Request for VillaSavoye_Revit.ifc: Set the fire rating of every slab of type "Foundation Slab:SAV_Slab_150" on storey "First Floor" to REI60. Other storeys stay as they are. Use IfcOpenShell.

First a look at what the model holds.

```python
import ifcopenshell
import ifcopenshell.util.element

model = ifcopenshell.open("VillaSavoye_Revit.ifc")
print(model.schema)
storey = next(s for s in model.by_type("IfcBuildingStorey") if s.Name == "First Floor")
slabs = [e for e in ifcopenshell.util.element.get_decomposition(storey) if e.is_a("IfcSlab")]
seen = {}
for e in slabs:
    element_type = ifcopenshell.util.element.get_type(e)
    key = (element_type.Name if element_type != e and element_type else None, ifcopenshell.util.element.get_pset(e, "Pset_SlabCommon", "FireRating"))
    seen[key] = seen.get(key, 0) + 1
for (name, value), count in sorted(seen.items(), key=str):
    print(count, "x", name, "|", value)
```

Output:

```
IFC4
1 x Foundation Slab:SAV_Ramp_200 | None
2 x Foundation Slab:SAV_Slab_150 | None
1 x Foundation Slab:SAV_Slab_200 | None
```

```python
import ifcopenshell
import ifcopenshell.api.pset
import ifcopenshell.util.element

model = ifcopenshell.open("VillaSavoye_Revit.ifc")

storey = next(s for s in model.by_type("IfcBuildingStorey") if s.Name == "First Floor")
slabs = [e for e in ifcopenshell.util.element.get_decomposition(storey) if e.is_a("IfcSlab")]

count = 0
for e in slabs:
    element_type = ifcopenshell.util.element.get_type(e)
    if element_type in (None, e) or element_type.Name != "Foundation Slab:SAV_Slab_150":
        continue
    # add_pset returns the element's existing set when there is one.
    pset = ifcopenshell.api.pset.add_pset(model, product=e, name="Pset_SlabCommon")
    ifcopenshell.api.pset.edit_pset(model, pset=pset, properties={"FireRating": "REI60"})
    count += 1

print(count, "slabs updated")

model.write("VillaSavoye_Revit_edited.ifc")
```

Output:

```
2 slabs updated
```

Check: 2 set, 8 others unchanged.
